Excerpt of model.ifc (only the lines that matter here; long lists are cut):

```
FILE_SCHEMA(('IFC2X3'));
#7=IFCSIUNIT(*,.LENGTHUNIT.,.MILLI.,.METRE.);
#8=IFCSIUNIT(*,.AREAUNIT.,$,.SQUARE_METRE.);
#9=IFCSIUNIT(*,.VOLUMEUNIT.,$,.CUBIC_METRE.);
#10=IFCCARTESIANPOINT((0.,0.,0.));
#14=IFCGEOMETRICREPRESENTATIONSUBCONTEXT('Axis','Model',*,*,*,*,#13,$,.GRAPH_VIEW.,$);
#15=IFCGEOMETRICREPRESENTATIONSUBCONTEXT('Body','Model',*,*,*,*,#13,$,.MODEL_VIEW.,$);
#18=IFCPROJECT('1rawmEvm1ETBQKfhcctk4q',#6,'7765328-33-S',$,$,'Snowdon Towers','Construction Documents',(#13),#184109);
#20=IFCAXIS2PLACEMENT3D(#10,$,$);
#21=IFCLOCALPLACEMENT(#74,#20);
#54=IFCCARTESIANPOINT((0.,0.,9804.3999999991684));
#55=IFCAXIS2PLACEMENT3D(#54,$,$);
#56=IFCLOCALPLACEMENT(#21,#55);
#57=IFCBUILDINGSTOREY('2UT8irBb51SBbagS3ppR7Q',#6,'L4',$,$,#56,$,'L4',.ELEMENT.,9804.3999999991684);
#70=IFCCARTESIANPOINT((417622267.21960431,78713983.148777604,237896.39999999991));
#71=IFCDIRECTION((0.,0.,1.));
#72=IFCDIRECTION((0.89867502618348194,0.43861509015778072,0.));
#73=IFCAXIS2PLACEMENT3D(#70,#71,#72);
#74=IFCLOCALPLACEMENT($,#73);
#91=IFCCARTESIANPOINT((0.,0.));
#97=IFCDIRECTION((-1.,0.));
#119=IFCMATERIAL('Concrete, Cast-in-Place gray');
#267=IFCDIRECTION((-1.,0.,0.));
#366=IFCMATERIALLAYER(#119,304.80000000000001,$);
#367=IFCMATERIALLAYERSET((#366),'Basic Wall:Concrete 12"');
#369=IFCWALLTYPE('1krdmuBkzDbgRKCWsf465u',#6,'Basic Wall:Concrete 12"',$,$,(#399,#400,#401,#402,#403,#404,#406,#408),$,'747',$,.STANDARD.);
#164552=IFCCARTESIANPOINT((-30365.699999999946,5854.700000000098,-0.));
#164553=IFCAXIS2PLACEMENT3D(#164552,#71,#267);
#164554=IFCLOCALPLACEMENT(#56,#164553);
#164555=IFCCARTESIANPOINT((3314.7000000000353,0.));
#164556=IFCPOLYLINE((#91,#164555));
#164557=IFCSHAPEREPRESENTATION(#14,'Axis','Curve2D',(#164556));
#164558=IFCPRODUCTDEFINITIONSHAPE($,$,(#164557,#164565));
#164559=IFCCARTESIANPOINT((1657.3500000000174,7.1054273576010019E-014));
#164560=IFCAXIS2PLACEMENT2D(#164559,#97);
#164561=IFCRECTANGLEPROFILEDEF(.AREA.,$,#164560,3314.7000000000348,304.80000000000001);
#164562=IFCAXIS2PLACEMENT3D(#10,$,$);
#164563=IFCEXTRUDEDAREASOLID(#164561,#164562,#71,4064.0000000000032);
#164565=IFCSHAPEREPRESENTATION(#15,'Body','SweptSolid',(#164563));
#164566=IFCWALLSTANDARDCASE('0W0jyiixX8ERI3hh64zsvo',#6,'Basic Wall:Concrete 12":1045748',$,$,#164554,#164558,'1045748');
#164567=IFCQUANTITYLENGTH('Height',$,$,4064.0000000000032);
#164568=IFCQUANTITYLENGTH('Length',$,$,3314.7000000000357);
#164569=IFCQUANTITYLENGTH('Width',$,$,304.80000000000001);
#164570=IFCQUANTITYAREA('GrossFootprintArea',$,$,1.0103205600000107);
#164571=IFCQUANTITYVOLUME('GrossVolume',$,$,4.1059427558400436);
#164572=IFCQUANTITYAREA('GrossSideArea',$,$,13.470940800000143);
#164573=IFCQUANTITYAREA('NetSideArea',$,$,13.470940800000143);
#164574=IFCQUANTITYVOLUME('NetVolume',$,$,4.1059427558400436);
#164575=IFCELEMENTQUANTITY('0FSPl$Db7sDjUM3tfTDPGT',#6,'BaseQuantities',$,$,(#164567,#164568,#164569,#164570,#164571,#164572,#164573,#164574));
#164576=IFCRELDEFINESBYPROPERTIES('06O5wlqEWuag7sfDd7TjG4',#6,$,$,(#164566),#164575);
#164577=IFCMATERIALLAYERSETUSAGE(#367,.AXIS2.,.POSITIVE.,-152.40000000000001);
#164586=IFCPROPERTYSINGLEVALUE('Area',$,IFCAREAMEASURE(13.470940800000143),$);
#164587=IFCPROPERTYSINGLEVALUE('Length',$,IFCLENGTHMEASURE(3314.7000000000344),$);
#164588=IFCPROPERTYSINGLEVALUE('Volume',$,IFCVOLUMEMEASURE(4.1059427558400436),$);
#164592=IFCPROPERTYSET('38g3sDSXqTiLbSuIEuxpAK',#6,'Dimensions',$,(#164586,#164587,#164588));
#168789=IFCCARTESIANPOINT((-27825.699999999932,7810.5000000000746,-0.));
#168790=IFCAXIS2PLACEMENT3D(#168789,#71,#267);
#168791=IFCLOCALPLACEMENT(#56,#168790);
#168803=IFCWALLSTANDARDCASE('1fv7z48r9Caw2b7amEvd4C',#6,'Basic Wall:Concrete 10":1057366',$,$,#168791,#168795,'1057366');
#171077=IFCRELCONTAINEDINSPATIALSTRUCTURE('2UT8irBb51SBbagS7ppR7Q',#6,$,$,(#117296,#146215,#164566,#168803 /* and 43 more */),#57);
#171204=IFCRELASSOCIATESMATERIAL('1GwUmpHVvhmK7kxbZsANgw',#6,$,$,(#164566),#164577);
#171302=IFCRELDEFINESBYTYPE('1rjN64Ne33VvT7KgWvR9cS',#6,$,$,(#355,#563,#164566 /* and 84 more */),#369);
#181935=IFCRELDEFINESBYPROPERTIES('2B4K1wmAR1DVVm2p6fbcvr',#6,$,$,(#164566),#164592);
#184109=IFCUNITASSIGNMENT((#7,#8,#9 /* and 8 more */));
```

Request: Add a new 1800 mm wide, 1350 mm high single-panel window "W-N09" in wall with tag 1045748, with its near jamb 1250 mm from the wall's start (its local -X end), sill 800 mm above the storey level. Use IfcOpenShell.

```python
import numpy as np
import ifcopenshell
import ifcopenshell.api.feature
import ifcopenshell.api.geometry
import ifcopenshell.api.pset
import ifcopenshell.api.root
import ifcopenshell.api.spatial
import ifcopenshell.api.type
import ifcopenshell.geom
import ifcopenshell.util.element
import ifcopenshell.util.placement
import ifcopenshell.util.representation
import ifcopenshell.util.shape
import ifcopenshell.util.unit

model = ifcopenshell.open("model.ifc")
unit_scale = ifcopenshell.util.unit.calculate_unit_scale(model)
area_scale = ifcopenshell.util.unit.calculate_unit_scale(model, "AREAUNIT")
volume_scale = ifcopenshell.util.unit.calculate_unit_scale(model, "VOLUMEUNIT")
settings = ifcopenshell.geom.settings()


def volume(element):
    """Net volume in cubic metres, openings subtracted."""
    shape = ifcopenshell.geom.create_shape(settings, element)
    return ifcopenshell.util.shape.get_volume(shape.geometry)


wall = model.by_guid("0W0jyiixX8ERI3hh64zsvo")
storey = ifcopenshell.util.element.get_container(wall, ifc_class="IfcBuildingStorey")
context = ifcopenshell.util.representation.get_context(model, "Model", "Body", "MODEL_VIEW")
before = volume(wall)

width, height, from_end, sill = 1.8, 1.35, 1.25, 0.8  # metres

# The wall runs along its own X axis, and the end named is its -X end.
wall_shape = ifcopenshell.geom.create_shape(settings, wall)
x, y, z = ifcopenshell.util.shape.get_vertices(wall_shape.geometry).T
start = x.min() + from_end
face, thickness = float(y.min()), float(y.max() - y.min())
wall_matrix = ifcopenshell.util.placement.get_local_placement(wall.ObjectPlacement)
level = ifcopenshell.util.placement.get_local_placement(storey.ObjectPlacement)[2, 3]


def in_wall(x, y):
    """Placement at x, y metres in the wall's axes, at sill height."""
    matrix = wall_matrix.copy()
    matrix[:, 3] = wall_matrix @ np.array([x / unit_scale, y / unit_scale, 0.0, 1.0])
    matrix[2, 3] = level + sill / unit_scale
    return matrix


# Opening: a box that overshoots both wall faces by 50 mm.
opening = ifcopenshell.api.root.create_entity(model, ifc_class="IfcOpeningElement")
box = ifcopenshell.api.geometry.add_wall_representation(
    model, context=context, length=width, height=height, thickness=thickness + 0.1
)
ifcopenshell.api.geometry.assign_representation(model, product=opening, representation=box)
ifcopenshell.api.geometry.edit_object_placement(model, product=opening, matrix=in_wall(start, face - 0.05), is_si=False)
ifcopenshell.api.feature.add_feature(model, feature=opening, element=wall)

window = ifcopenshell.api.root.create_entity(model, ifc_class="IfcWindow", name="W-N09")
window.OverallWidth, window.OverallHeight = width / unit_scale, height / unit_scale
body = ifcopenshell.api.geometry.add_window_representation(
    model,
    context=context,
    overall_width=window.OverallWidth,
    overall_height=window.OverallHeight,
    partition_type="SINGLE_PANEL",
)
ifcopenshell.api.geometry.assign_representation(model, product=window, representation=body)
ifcopenshell.api.spatial.assign_container(model, products=[window], relating_structure=storey)
fills = ifcopenshell.api.feature.add_filling(model, opening=opening, element=window)
fills.OwnerHistory = window.OwnerHistory  # required in IFC2X3

# IFC2X3 keeps the operation on the window style.
style = ifcopenshell.api.root.create_entity(model, ifc_class="IfcWindowStyle", name="W-N09")
style.OperationType, style.ConstructionType = "SINGLE_PANEL", "NOTDEFINED"
style.ParameterTakesPrecedence = style.Sizeable = False
ifcopenshell.api.type.assign_type(model, related_objects=[window], relating_type=style)

# Centre the window in the wall's thickness.
ifcopenshell.api.geometry.edit_object_placement(model, product=window, matrix=in_wall(start, face), is_si=False)
window_shape = ifcopenshell.geom.create_shape(settings, window)
depth = ifcopenshell.util.shape.get_vertices(window_shape.geometry)[:, 1]
offset = face + thickness / 2 - (depth.min() + depth.max()) / 2
ifcopenshell.api.geometry.edit_object_placement(model, product=window, matrix=in_wall(start, offset), is_si=False)

after = volume(wall)

# Update the wall's stored quantities.
qto = model.by_id(ifcopenshell.util.element.get_pset(wall, "BaseQuantities", should_inherit=False)["id"])
ifcopenshell.api.pset.edit_qto(model, qto=qto, properties={
    "NetSideArea": after / thickness / area_scale,
    "NetVolume": after / volume_scale,
})
pset = model.by_id(ifcopenshell.util.element.get_pset(wall, "Dimensions", should_inherit=False)["id"])
ifcopenshell.api.pset.edit_pset(model, pset=pset, properties={
    "Area": model.create_entity("IfcAreaMeasure", after / thickness / area_scale),
    "Volume": model.create_entity("IfcVolumeMeasure", after / volume_scale),
})

print(f"wall volume {before:.3f} -> {after:.3f} m3")

model.write("model-out.ifc")
```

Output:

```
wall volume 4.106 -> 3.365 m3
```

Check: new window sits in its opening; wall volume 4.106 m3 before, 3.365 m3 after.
